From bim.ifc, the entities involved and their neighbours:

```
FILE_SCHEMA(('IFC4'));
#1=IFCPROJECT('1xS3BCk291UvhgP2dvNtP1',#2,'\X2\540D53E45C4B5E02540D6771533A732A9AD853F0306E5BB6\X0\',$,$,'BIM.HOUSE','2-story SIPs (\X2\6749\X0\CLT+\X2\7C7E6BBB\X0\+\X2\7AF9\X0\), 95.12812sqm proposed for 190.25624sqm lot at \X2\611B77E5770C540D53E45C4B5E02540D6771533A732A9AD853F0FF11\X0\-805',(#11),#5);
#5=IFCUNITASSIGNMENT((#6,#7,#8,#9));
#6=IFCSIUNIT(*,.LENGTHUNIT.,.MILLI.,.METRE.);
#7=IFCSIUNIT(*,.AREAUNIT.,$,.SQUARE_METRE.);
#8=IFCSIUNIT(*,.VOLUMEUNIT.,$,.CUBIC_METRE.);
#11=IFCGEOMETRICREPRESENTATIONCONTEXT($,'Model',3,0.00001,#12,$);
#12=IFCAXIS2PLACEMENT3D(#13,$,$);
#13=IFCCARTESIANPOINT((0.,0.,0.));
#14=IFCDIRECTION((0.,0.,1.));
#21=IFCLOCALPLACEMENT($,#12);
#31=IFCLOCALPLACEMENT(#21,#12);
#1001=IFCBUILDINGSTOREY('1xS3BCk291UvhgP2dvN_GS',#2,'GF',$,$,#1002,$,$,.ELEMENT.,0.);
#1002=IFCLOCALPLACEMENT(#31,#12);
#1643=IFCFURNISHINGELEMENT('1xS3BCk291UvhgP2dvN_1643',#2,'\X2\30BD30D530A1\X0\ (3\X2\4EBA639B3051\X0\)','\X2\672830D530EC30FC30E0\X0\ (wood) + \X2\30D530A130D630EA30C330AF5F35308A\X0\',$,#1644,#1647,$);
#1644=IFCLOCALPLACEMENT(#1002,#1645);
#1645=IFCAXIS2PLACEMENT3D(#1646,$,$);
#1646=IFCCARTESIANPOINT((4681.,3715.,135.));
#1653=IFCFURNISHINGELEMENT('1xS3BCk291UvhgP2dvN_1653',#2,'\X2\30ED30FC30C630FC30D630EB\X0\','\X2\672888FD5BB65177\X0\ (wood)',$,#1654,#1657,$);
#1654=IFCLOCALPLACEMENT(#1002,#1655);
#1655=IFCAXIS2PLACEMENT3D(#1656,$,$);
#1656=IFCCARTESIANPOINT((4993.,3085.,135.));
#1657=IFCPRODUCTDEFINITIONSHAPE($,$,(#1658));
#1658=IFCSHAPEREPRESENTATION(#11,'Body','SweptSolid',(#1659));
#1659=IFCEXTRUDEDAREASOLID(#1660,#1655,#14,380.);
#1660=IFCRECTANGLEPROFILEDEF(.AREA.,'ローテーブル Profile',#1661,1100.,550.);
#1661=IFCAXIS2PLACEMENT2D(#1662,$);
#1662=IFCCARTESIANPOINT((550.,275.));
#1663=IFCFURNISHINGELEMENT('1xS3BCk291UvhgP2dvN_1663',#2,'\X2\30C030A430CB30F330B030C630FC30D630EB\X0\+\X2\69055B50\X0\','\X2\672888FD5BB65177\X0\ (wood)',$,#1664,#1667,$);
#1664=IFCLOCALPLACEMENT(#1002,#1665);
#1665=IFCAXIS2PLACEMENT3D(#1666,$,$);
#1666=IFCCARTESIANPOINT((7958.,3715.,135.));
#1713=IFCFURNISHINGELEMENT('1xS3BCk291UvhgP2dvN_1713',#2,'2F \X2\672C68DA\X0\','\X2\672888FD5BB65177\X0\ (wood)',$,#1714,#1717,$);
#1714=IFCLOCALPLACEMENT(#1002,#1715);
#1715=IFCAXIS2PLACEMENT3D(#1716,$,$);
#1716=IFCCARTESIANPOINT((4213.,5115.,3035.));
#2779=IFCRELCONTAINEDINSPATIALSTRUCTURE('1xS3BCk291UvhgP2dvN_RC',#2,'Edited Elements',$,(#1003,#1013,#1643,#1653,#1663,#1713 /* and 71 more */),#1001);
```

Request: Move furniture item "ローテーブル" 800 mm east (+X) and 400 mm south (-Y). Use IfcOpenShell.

```python
import ifcopenshell
import ifcopenshell.api.geometry
import ifcopenshell.util.placement

model = ifcopenshell.open("bim.ifc")

item = model.by_id(1653)
matrix = ifcopenshell.util.placement.get_local_placement(item.ObjectPlacement)
matrix[0, 3] += 800.0
matrix[1, 3] -= 400.0
ifcopenshell.api.geometry.edit_object_placement(model, product=item, matrix=matrix, is_si=False)

print(ifcopenshell.util.placement.get_local_placement(item.ObjectPlacement).round(3) + 0.0)

model.write("bim_updated.ifc")
```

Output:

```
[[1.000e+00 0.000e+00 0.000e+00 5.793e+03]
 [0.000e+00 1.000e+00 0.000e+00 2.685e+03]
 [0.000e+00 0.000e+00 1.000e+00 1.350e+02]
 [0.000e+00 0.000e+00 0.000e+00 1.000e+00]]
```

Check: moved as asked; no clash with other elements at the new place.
